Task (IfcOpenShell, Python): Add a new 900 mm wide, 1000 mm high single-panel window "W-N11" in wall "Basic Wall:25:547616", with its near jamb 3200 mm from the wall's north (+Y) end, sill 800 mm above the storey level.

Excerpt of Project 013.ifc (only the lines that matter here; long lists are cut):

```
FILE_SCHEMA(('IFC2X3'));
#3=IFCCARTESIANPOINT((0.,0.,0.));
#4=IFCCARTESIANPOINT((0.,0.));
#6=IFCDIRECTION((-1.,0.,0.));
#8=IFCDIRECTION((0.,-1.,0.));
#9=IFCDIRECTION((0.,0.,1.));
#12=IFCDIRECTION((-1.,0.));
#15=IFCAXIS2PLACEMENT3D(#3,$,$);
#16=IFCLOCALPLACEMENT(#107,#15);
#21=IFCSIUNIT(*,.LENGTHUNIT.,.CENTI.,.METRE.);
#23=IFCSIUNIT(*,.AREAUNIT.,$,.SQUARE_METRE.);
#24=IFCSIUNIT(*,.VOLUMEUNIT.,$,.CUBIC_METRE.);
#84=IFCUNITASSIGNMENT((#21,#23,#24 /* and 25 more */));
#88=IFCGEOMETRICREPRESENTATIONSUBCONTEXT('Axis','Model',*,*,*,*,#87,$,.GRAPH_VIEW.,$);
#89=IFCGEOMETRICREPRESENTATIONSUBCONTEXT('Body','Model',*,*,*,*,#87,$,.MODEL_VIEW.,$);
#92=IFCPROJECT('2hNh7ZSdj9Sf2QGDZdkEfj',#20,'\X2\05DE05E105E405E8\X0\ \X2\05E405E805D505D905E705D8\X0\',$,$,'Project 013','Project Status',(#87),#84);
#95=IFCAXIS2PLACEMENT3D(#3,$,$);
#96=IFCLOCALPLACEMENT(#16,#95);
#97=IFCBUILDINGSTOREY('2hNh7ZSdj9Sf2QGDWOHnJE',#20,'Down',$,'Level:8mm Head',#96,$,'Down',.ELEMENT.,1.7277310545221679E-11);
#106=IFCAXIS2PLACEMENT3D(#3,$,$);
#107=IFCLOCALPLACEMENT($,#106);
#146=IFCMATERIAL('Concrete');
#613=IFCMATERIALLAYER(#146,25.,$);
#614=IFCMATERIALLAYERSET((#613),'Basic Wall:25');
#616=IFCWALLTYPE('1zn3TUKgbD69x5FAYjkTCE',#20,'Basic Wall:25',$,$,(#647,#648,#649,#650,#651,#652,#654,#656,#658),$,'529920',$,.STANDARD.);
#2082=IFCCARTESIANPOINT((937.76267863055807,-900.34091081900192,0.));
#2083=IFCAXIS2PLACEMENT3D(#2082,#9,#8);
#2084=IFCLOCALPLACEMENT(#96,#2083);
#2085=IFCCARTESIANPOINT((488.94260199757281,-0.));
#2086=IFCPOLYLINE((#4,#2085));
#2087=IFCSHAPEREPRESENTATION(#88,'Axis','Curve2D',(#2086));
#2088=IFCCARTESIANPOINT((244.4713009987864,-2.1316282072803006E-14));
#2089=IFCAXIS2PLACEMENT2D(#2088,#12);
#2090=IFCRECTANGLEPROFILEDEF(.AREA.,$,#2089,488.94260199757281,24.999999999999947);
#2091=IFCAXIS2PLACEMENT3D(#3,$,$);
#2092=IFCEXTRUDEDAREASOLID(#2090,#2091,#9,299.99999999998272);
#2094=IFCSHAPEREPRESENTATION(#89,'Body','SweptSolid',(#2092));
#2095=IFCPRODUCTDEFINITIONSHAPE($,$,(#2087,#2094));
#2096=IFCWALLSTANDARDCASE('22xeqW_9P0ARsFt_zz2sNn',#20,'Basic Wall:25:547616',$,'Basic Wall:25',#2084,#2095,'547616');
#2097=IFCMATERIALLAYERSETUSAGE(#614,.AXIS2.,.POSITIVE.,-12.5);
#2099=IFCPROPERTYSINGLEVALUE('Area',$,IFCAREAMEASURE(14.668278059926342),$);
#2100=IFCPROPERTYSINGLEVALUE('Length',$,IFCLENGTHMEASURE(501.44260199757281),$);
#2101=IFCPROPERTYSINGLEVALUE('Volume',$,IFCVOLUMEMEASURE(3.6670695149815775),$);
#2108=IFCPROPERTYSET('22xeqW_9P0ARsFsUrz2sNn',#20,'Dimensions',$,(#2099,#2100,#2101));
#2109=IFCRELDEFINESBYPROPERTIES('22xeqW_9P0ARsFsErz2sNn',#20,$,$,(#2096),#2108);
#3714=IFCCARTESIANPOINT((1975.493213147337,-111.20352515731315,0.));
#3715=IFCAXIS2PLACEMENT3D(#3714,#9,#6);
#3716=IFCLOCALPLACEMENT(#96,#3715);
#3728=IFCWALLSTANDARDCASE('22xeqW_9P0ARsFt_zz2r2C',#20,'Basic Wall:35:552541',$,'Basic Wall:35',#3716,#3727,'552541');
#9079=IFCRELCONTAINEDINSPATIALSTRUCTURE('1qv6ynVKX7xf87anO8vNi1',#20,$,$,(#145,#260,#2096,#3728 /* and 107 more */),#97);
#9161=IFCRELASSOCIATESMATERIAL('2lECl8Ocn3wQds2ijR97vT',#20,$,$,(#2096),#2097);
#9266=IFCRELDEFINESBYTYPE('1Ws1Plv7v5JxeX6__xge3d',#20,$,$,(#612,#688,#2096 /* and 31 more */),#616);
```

```python
import numpy as np
import ifcopenshell
import ifcopenshell.api.feature
import ifcopenshell.api.geometry
import ifcopenshell.api.pset
import ifcopenshell.api.root
import ifcopenshell.api.spatial
import ifcopenshell.api.type
import ifcopenshell.geom
import ifcopenshell.util.element
import ifcopenshell.util.placement
import ifcopenshell.util.representation
import ifcopenshell.util.shape
import ifcopenshell.util.unit

model = ifcopenshell.open("Project 013.ifc")
unit_scale = ifcopenshell.util.unit.calculate_unit_scale(model)
area_scale = ifcopenshell.util.unit.calculate_unit_scale(model, "AREAUNIT")
volume_scale = ifcopenshell.util.unit.calculate_unit_scale(model, "VOLUMEUNIT")
settings = ifcopenshell.geom.settings()


def volume(element):
    """Net volume in cubic metres, openings subtracted."""
    shape = ifcopenshell.geom.create_shape(settings, element)
    return ifcopenshell.util.shape.get_volume(shape.geometry)


wall = model.by_id(2096)
storey = ifcopenshell.util.element.get_container(wall, ifc_class="IfcBuildingStorey")
context = ifcopenshell.util.representation.get_context(model, "Model", "Body", "MODEL_VIEW")
before = volume(wall)

width, height, from_end, sill = 0.9, 1, 3.2, 0.8  # metres

# The wall runs along its own X axis, and the end named is its -X end.
wall_shape = ifcopenshell.geom.create_shape(settings, wall)
x, y, z = ifcopenshell.util.shape.get_vertices(wall_shape.geometry).T
start = x.min() + from_end
face, thickness = float(y.min()), float(y.max() - y.min())
wall_matrix = ifcopenshell.util.placement.get_local_placement(wall.ObjectPlacement)
level = ifcopenshell.util.placement.get_local_placement(storey.ObjectPlacement)[2, 3]


def in_wall(x, y):
    """Placement at x, y metres in the wall's axes, at sill height."""
    matrix = wall_matrix.copy()
    matrix[:, 3] = wall_matrix @ np.array([x / unit_scale, y / unit_scale, 0.0, 1.0])
    matrix[2, 3] = level + sill / unit_scale
    return matrix


# Opening: a box that overshoots both wall faces by 50 mm.
opening = ifcopenshell.api.root.create_entity(model, ifc_class="IfcOpeningElement")
box = ifcopenshell.api.geometry.add_wall_representation(
    model, context=context, length=width, height=height, thickness=thickness + 0.1
)
ifcopenshell.api.geometry.assign_representation(model, product=opening, representation=box)
ifcopenshell.api.geometry.edit_object_placement(model, product=opening, matrix=in_wall(start, face - 0.05), is_si=False)
ifcopenshell.api.feature.add_feature(model, feature=opening, element=wall)

window = ifcopenshell.api.root.create_entity(model, ifc_class="IfcWindow", name="W-N11")
window.OverallWidth, window.OverallHeight = width / unit_scale, height / unit_scale
body = ifcopenshell.api.geometry.add_window_representation(
    model,
    context=context,
    overall_width=window.OverallWidth,
    overall_height=window.OverallHeight,
    partition_type="SINGLE_PANEL",
)
ifcopenshell.api.geometry.assign_representation(model, product=window, representation=body)
ifcopenshell.api.spatial.assign_container(model, products=[window], relating_structure=storey)
fills = ifcopenshell.api.feature.add_filling(model, opening=opening, element=window)
fills.OwnerHistory = window.OwnerHistory  # required in IFC2X3

# IFC2X3 keeps the operation on the window style.
style = ifcopenshell.api.root.create_entity(model, ifc_class="IfcWindowStyle", name="W-N11")
style.OperationType, style.ConstructionType = "SINGLE_PANEL", "NOTDEFINED"
style.ParameterTakesPrecedence = style.Sizeable = False
ifcopenshell.api.type.assign_type(model, related_objects=[window], relating_type=style)

# Centre the window in the wall's thickness.
ifcopenshell.api.geometry.edit_object_placement(model, product=window, matrix=in_wall(start, face), is_si=False)
window_shape = ifcopenshell.geom.create_shape(settings, window)
depth = ifcopenshell.util.shape.get_vertices(window_shape.geometry)[:, 1]
offset = face + thickness / 2 - (depth.min() + depth.max()) / 2
ifcopenshell.api.geometry.edit_object_placement(model, product=window, matrix=in_wall(start, offset), is_si=False)

after = volume(wall)

# Update the wall's stored quantities.
pset = model.by_id(ifcopenshell.util.element.get_pset(wall, "Dimensions", should_inherit=False)["id"])
ifcopenshell.api.pset.edit_pset(model, pset=pset, properties={
    "Area": model.create_entity("IfcAreaMeasure", after / thickness / area_scale),
    "Volume": model.create_entity("IfcVolumeMeasure", after / volume_scale),
})

print(f"wall volume {before:.3f} -> {after:.3f} m3")

model.write("Project 013-out.ifc")
```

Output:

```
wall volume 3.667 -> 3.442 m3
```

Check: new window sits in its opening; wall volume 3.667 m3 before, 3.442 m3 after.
